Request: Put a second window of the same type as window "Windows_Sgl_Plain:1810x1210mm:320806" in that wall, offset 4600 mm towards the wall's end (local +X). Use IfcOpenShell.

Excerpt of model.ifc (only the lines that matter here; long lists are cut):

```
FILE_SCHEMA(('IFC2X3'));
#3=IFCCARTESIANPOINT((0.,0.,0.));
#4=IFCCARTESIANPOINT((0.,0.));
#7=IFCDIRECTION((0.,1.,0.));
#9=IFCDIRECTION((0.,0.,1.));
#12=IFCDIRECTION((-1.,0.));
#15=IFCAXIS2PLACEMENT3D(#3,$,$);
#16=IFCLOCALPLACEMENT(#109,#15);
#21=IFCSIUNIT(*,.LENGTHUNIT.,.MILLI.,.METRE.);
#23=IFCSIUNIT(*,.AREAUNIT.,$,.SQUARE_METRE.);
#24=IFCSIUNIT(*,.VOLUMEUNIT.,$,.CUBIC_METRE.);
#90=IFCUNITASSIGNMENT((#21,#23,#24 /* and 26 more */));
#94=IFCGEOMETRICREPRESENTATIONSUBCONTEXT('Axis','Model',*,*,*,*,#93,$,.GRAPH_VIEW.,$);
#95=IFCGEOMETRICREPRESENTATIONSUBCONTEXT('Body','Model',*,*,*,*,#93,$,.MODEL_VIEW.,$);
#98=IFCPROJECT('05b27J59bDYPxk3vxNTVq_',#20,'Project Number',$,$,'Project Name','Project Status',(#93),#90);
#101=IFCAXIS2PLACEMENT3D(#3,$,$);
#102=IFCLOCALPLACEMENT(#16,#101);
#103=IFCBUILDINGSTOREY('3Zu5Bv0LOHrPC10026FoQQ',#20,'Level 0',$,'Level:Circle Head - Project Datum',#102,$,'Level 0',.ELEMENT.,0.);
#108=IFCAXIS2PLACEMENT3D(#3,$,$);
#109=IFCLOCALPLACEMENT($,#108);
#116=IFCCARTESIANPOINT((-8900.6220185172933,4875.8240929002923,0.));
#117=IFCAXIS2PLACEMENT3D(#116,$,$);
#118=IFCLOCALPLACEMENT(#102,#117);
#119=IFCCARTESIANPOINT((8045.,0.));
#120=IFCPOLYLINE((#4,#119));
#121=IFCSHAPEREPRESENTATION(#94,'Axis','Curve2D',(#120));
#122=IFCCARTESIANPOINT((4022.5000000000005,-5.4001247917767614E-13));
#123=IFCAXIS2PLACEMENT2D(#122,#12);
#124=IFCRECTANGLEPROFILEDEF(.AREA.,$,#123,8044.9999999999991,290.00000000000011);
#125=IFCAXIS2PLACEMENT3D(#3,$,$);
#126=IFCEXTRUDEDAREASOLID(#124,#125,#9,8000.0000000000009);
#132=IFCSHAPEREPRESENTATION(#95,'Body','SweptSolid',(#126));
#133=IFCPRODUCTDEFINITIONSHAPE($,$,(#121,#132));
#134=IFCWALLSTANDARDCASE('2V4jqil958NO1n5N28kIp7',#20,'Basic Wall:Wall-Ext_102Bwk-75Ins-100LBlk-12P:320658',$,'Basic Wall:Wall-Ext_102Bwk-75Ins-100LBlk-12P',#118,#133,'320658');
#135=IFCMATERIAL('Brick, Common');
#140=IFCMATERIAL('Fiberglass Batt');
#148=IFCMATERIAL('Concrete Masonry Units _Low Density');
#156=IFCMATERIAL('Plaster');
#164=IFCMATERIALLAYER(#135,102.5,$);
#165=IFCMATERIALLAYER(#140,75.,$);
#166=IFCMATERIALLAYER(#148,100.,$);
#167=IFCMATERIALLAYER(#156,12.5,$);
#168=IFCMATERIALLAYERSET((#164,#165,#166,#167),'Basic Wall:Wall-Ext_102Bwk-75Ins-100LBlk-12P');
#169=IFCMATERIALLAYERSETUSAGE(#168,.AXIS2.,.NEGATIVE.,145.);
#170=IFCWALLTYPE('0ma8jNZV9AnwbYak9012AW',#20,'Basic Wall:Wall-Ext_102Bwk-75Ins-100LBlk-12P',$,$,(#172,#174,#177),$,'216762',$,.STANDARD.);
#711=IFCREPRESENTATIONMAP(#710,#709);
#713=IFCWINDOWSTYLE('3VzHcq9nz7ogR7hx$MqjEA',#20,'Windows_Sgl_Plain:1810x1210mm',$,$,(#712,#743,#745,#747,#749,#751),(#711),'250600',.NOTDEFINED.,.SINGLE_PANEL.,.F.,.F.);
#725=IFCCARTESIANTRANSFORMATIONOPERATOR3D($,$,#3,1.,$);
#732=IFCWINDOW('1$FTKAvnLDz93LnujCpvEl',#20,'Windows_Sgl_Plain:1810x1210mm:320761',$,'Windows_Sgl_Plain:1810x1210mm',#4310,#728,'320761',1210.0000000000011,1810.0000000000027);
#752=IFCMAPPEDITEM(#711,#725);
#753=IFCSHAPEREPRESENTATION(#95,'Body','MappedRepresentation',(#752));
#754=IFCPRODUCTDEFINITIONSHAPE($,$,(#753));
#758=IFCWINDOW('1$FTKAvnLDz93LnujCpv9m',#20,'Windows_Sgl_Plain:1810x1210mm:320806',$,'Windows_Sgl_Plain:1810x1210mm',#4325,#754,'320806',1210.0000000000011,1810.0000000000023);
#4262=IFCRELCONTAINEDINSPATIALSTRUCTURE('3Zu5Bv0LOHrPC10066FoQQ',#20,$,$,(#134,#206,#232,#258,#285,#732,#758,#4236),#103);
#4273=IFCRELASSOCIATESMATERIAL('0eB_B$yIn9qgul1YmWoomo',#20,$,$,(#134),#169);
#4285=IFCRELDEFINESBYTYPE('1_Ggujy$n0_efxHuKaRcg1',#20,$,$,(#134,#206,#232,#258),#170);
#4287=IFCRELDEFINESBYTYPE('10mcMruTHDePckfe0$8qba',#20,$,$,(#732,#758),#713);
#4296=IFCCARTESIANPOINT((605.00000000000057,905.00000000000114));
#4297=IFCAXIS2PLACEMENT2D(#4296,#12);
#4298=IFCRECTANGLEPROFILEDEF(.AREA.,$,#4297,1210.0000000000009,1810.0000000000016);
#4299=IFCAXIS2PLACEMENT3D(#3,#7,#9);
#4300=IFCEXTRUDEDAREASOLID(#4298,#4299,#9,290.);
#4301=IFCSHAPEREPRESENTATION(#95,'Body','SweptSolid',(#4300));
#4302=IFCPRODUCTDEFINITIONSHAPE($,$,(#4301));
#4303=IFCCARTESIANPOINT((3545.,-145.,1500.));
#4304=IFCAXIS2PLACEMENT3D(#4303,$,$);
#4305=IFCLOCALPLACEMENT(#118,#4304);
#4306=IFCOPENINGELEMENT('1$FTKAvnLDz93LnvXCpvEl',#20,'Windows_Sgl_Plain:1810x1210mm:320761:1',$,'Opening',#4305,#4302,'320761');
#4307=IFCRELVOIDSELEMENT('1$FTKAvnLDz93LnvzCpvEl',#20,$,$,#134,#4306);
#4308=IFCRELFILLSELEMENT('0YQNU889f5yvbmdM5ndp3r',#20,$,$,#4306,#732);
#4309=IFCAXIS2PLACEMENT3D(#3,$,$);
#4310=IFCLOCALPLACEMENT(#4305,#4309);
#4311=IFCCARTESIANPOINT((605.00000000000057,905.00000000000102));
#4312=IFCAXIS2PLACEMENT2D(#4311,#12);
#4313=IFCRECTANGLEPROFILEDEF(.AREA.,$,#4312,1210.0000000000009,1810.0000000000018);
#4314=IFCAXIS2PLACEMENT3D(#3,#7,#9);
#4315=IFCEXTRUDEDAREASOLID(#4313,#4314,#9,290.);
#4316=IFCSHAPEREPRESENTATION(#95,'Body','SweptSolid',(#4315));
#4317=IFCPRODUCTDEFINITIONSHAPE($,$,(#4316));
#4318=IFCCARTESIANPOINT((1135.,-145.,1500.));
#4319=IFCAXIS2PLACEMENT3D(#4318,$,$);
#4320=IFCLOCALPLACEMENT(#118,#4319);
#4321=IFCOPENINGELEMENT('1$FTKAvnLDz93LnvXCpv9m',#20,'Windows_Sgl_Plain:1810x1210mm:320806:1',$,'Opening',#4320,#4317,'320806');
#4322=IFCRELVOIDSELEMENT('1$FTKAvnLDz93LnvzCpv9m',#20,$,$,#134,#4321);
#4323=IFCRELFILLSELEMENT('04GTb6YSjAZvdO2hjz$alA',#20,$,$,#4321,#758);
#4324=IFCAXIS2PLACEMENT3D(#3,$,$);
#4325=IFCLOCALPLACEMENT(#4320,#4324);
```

```python
import ifcopenshell
import ifcopenshell.api.feature
import ifcopenshell.api.geometry
import ifcopenshell.api.root
import ifcopenshell.geom
import ifcopenshell.util.element
import ifcopenshell.util.placement
import ifcopenshell.util.shape

model = ifcopenshell.open("model.ifc")
settings = ifcopenshell.geom.settings()


def volume(element):
    """Net volume in cubic metres, openings subtracted."""
    shape = ifcopenshell.geom.create_shape(settings, element)
    return ifcopenshell.util.shape.get_volume(shape.geometry)


def reuse_history(source, copy):
    """copy_class also copies each property set's owner history, people and application; keep the originals."""
    for rel in copy.IsDefinedBy:
        if rel.is_a("IfcRelDefinesByProperties") and (history := rel.RelatingPropertyDefinition.OwnerHistory):
            rel.RelatingPropertyDefinition.OwnerHistory = source.OwnerHistory
            ifcopenshell.util.element.remove_deep2(model, history)


window = model.by_id(758)
opening = window.FillsVoids[0].RelatingOpeningElement
wall = opening.VoidsElements[0].RelatingBuildingElement
before = volume(wall)
shift = ifcopenshell.util.placement.get_local_placement(wall.ObjectPlacement)[:3, 0] * 4600.0

# copy_class copies the void relationship, type, container and properties, but no geometry.
new_opening = ifcopenshell.api.root.copy_class(model, product=opening)
new_opening.Representation = ifcopenshell.util.element.copy_deep(
    model, opening.Representation, exclude=["IfcGeometricRepresentationContext", "IfcRepresentationMap"]
)
new_opening.Name = "Windows_Sgl_Plain:1810x1210mm"
new_opening.Tag = None
new_window = ifcopenshell.api.root.copy_class(model, product=window)
new_window.Representation = ifcopenshell.util.element.copy_deep(
    model, window.Representation, exclude=["IfcGeometricRepresentationContext", "IfcRepresentationMap"]
)
new_window.Name = "Windows_Sgl_Plain:1810x1210mm"
new_window.Tag = None
reuse_history(window, new_window)
fills = ifcopenshell.api.feature.add_filling(model, opening=new_opening, element=new_window)
fills.OwnerHistory = new_window.OwnerHistory  # required in IFC2X3

for old, new in ((opening, new_opening), (window, new_window)):
    matrix = ifcopenshell.util.placement.get_local_placement(old.ObjectPlacement)
    matrix[:3, 3] += shift
    ifcopenshell.api.geometry.edit_object_placement(model, product=new, matrix=matrix, is_si=False)

after = volume(wall)

print(f"wall volume {before:.3f} -> {after:.3f} m3")

model.write("model_rev.ifc")
```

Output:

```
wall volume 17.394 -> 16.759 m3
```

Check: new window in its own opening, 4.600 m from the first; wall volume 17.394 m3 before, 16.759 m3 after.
